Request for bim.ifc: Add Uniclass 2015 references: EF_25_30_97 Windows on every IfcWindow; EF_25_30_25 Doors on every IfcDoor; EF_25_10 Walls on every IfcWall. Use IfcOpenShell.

First a look at what the model holds.

```python
import ifcopenshell

model = ifcopenshell.open("bim.ifc")
print(model.schema)
print("classifications:", [c.Name for c in model.by_type("IfcClassification")])
for ifc_class in ("IfcDoor", "IfcRoof", "IfcStair", "IfcWall", "IfcWindow"):
    print(ifc_class, len(model.by_type(ifc_class)))
```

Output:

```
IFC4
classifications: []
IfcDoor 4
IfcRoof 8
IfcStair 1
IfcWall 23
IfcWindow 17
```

```python
import ifcopenshell
import ifcopenshell.api.classification

model = ifcopenshell.open("bim.ifc")

system = ifcopenshell.api.classification.add_classification(model, classification="Uniclass 2015")

codes = {
    "IfcWindow": ("EF_25_30_97", "Windows"),
    "IfcDoor": ("EF_25_30_25", "Doors"),
    "IfcWall": ("EF_25_10", "Walls"),
}
for ifc_class, (code, name) in codes.items():
    products = model.by_type(ifc_class)
    ifcopenshell.api.classification.add_reference(
        model, products=products, classification=system, identification=code, name=name
    )
    print(code, len(products))

model.write("bim_v2.ifc")
```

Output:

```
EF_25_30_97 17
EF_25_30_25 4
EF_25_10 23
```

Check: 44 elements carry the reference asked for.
